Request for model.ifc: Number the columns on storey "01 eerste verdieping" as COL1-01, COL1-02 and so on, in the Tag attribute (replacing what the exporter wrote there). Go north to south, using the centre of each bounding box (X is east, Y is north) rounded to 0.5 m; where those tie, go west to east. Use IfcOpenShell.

First a look at what the model holds.

```python
import ifcopenshell
import ifcopenshell.util.element
import ifcopenshell.util.placement

model = ifcopenshell.open("model.ifc")
print(model.schema)
storey = next(s for s in model.by_type("IfcBuildingStorey") if s.Name == "01 eerste verdieping")
columns = [e for e in ifcopenshell.util.element.get_decomposition(storey) if e.is_a("IfcColumn")]
for e in sorted(columns, key=lambda e: e.id()):
    origin = ifcopenshell.util.placement.get_local_placement(e.ObjectPlacement)[:3, 3]
    print(e.id(), e.Tag, e.Name, origin.round(2) + 0.0, sep=" | ")
```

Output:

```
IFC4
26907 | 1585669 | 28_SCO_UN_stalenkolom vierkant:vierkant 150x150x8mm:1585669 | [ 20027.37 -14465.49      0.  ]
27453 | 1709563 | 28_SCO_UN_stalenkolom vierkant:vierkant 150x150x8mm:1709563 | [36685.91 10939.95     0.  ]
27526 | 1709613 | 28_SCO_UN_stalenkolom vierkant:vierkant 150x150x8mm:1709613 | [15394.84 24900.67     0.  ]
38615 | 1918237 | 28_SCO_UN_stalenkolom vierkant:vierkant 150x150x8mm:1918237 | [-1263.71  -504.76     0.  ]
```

```python
import ifcopenshell
import ifcopenshell.geom
import ifcopenshell.util.element
import ifcopenshell.util.shape

model = ifcopenshell.open("model.ifc")
settings = ifcopenshell.geom.settings()
settings.set("use-world-coords", True)


def centre(element):
    shape = ifcopenshell.geom.create_shape(settings, element)
    return ifcopenshell.util.shape.get_bbox_centroid(shape.geometry)


storey = next(s for s in model.by_type("IfcBuildingStorey") if s.Name == "01 eerste verdieping")
columns = [e for e in ifcopenshell.util.element.get_decomposition(storey) if e.is_a("IfcColumn")]

# Insertion points can sit at a corner or the storey origin, so sort by the geometry (in metres).
centres = {e: centre(e) for e in columns}
columns.sort(key=lambda e: (-round(centres[e][1] / 0.5), centres[e][0]))

for i, e in enumerate(columns, start=1):
    number = f"COL1-{i:02d}"
    e.Tag = number
    print(e.id(), number)

model.write("model_rev.ifc")
```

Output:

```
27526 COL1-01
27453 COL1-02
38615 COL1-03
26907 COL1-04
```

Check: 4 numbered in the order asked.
